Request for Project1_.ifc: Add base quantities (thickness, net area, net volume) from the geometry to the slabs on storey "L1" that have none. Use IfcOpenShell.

First a look at what the model holds.

```python
import ifcopenshell
import ifcopenshell.util.element
import ifcopenshell.util.unit

model = ifcopenshell.open("Project1_.ifc")
print(model.schema)
for unit_type in ("LENGTHUNIT", "AREAUNIT", "VOLUMEUNIT"):
    print(unit_type, ifcopenshell.util.unit.calculate_unit_scale(model, unit_type))
storey = next(s for s in model.by_type("IfcBuildingStorey") if s.Name == "L1")
slabs = [e for e in ifcopenshell.util.element.get_decomposition(storey) if e.is_a("IfcSlab")]
for e in sorted(slabs, key=lambda e: e.id()):
    print(e.id(), e.is_a(), e.Name, list(ifcopenshell.util.element.get_psets(e, qtos_only=True)), sep=" | ")
```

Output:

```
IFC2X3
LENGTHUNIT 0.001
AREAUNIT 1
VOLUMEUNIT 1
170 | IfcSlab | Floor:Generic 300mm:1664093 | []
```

```python
import ifcopenshell
import ifcopenshell.api.pset
import ifcopenshell.geom
import ifcopenshell.util.element
import ifcopenshell.util.shape
import ifcopenshell.util.unit

model = ifcopenshell.open("Project1_.ifc")
unit_scale = ifcopenshell.util.unit.calculate_unit_scale(model)
area_scale = ifcopenshell.util.unit.calculate_unit_scale(model, "AREAUNIT")
volume_scale = ifcopenshell.util.unit.calculate_unit_scale(model, "VOLUMEUNIT")
settings = ifcopenshell.geom.settings()

storey = next(s for s in model.by_type("IfcBuildingStorey") if s.Name == "L1")
slabs = [e for e in ifcopenshell.util.element.get_decomposition(storey) if e.is_a("IfcSlab")]

for e in sorted(slabs, key=lambda e: e.id()):
    if ifcopenshell.util.element.get_psets(e, qtos_only=True, should_inherit=False):
        continue
    # Geometry comes back in metres, in the element's own axes.
    shape = ifcopenshell.geom.create_shape(settings, e)
    values = {
        "Width": ifcopenshell.util.shape.get_z(shape.geometry) / unit_scale,
        "NetArea": ifcopenshell.util.shape.get_footprint_area(shape.geometry) / area_scale,
        "NetVolume": ifcopenshell.util.shape.get_volume(shape.geometry) / volume_scale,
    }
    qto = ifcopenshell.api.pset.add_qto(model, product=e, name="BaseQuantities")
    ifcopenshell.api.pset.edit_qto(model, qto=qto, properties=values)
    print(e.id(), {k: round(v, 3) for k, v in values.items()})

model.write("Project1_-out.ifc")
```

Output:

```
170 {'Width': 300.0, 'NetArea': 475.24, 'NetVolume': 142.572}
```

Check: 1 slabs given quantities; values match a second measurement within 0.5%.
